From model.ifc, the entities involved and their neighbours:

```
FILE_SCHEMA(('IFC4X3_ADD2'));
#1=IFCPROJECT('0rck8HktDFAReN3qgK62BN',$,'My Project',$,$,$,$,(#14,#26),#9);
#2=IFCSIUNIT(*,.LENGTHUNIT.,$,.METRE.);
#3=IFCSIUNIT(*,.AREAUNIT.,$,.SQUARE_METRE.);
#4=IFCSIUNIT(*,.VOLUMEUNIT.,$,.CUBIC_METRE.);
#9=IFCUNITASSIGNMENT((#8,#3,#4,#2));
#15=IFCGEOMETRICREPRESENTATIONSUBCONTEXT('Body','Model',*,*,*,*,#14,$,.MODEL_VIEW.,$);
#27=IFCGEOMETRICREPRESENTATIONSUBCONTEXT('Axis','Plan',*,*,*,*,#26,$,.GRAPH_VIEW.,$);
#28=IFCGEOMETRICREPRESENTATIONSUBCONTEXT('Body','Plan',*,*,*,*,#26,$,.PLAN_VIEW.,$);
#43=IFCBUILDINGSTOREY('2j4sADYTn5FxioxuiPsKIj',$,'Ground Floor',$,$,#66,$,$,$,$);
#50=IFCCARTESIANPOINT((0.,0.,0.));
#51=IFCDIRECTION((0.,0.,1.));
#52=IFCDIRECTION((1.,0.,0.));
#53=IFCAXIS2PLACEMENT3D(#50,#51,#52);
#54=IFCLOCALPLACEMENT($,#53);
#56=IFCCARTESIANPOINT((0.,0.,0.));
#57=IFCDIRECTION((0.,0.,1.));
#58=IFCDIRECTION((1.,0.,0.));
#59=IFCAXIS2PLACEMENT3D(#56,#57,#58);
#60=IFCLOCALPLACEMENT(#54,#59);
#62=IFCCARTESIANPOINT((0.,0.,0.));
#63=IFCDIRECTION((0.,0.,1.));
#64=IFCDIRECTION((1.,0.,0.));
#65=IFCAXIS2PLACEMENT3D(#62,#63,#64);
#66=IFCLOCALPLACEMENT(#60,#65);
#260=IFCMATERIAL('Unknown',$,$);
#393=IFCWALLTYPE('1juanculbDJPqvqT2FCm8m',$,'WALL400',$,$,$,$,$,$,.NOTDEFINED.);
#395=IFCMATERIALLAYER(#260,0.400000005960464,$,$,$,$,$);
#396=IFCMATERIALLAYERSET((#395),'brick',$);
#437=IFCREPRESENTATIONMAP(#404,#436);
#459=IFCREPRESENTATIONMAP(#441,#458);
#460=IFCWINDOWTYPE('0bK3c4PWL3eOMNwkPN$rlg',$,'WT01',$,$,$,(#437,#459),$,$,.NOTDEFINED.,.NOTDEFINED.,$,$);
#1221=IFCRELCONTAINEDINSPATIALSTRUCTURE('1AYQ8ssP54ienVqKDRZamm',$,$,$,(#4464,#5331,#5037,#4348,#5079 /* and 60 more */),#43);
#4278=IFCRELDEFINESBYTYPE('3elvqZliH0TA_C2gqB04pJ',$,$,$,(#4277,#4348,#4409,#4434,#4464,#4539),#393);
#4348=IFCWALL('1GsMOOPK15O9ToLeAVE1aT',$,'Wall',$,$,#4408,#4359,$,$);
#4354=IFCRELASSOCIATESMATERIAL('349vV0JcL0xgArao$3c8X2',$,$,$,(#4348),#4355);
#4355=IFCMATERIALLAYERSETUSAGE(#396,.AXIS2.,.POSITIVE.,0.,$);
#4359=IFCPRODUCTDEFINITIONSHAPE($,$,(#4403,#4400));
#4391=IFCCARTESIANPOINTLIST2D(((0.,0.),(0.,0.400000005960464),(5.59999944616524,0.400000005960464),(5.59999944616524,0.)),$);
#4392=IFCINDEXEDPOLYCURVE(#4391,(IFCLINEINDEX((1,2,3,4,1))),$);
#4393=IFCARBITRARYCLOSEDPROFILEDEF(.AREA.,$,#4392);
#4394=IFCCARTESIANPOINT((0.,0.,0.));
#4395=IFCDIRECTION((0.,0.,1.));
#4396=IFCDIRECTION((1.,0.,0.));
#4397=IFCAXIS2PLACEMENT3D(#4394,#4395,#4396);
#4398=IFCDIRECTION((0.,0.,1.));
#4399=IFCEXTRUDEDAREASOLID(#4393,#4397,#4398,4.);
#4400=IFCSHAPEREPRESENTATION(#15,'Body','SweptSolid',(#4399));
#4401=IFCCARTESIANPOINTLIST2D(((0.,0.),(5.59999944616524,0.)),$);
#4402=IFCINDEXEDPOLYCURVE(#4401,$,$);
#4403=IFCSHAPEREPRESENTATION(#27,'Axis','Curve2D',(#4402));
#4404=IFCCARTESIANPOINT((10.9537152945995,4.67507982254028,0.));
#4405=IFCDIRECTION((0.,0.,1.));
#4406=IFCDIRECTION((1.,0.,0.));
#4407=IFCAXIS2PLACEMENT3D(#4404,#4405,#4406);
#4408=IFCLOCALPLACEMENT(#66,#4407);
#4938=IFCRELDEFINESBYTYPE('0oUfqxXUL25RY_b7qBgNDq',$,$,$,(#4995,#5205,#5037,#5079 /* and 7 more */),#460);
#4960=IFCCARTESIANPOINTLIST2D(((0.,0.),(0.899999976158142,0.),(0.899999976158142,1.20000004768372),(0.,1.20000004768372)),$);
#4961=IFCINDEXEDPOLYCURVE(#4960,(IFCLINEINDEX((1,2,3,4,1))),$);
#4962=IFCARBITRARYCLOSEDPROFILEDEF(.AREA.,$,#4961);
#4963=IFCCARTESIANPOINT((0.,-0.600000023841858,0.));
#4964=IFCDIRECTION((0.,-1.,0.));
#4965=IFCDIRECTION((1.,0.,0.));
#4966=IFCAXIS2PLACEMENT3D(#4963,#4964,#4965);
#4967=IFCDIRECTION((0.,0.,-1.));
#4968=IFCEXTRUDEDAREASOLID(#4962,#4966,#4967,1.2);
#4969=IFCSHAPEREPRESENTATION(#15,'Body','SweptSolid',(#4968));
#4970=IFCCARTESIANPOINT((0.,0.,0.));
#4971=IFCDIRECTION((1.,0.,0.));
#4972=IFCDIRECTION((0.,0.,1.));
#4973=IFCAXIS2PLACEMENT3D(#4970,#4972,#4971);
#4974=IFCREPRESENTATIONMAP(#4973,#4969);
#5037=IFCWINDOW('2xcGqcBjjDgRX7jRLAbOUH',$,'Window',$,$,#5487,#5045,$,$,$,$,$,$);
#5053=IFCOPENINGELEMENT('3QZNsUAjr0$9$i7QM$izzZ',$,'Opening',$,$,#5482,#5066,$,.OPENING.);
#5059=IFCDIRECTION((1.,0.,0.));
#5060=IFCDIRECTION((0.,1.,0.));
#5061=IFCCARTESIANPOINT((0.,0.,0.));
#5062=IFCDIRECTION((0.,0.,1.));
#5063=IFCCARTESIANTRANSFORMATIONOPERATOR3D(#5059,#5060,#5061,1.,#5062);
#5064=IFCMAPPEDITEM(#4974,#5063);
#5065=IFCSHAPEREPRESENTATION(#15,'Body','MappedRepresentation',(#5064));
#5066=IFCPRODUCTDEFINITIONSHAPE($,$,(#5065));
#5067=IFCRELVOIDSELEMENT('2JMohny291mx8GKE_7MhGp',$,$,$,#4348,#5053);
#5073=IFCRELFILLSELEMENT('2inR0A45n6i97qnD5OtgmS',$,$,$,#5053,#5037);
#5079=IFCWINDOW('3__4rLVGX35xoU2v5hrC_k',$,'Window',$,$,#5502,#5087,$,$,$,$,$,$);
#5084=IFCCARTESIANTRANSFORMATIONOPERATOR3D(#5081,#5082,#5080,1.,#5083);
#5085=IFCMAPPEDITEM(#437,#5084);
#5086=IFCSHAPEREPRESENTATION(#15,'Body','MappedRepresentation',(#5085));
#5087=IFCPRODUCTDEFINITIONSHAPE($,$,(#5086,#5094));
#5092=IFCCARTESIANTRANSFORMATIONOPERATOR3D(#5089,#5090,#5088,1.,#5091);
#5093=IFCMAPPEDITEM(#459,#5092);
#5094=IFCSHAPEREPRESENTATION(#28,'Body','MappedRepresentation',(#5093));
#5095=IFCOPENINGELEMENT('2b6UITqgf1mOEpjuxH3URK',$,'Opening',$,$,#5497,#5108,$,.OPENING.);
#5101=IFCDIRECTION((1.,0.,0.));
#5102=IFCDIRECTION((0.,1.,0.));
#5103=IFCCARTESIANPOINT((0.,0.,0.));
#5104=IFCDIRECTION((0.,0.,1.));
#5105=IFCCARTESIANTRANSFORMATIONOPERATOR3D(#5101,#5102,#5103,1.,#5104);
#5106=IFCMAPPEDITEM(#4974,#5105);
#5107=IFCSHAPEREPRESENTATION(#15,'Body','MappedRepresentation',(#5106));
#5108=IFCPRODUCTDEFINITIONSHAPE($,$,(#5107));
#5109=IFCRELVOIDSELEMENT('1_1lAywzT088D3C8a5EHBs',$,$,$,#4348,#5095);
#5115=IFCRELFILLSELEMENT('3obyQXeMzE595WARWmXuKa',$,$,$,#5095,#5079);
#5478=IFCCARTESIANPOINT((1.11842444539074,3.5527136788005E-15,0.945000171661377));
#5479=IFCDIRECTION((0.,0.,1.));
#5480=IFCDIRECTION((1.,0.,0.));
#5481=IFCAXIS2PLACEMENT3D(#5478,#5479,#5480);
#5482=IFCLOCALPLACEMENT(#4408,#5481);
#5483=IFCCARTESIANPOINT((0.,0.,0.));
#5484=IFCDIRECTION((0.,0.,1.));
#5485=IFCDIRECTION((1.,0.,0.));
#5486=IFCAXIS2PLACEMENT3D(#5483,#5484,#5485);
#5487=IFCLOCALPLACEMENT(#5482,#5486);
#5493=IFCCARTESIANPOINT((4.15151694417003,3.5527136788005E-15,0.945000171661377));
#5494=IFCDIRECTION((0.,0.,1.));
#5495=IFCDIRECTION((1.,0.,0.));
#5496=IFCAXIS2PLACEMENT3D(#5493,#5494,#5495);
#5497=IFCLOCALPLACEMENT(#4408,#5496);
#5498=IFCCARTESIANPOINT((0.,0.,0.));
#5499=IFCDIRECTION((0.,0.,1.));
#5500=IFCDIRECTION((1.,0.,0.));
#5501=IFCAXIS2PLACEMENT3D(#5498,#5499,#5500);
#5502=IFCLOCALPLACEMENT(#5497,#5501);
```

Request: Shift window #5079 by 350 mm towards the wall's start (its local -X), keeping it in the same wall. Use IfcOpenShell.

```python
import ifcopenshell
import ifcopenshell.api.geometry
import ifcopenshell.util.placement

model = ifcopenshell.open("model.ifc")

window = model.by_id(5079)
opening = window.FillsVoids[0].RelatingOpeningElement
wall = opening.VoidsElements[0].RelatingBuildingElement

wall_matrix = ifcopenshell.util.placement.get_local_placement(wall.ObjectPlacement)
shift = wall_matrix[:3, 0] * -0.35
before = ifcopenshell.util.placement.get_local_placement(window.ObjectPlacement)[:3, 3].copy()

# The window is placed relative to its opening, so it follows when the opening moves.
matrix = ifcopenshell.util.placement.get_local_placement(opening.ObjectPlacement)
matrix[:3, 3] += shift
ifcopenshell.api.geometry.edit_object_placement(
    model, product=opening, matrix=matrix, is_si=False, should_transform_children=True
)

after = ifcopenshell.util.placement.get_local_placement(window.ObjectPlacement)[:3, 3]
print("window moved by", (after - before).round(3) + 0.0)

model.write("model_updated.ifc")
```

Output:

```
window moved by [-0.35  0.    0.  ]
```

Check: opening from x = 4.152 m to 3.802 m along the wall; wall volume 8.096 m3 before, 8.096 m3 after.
